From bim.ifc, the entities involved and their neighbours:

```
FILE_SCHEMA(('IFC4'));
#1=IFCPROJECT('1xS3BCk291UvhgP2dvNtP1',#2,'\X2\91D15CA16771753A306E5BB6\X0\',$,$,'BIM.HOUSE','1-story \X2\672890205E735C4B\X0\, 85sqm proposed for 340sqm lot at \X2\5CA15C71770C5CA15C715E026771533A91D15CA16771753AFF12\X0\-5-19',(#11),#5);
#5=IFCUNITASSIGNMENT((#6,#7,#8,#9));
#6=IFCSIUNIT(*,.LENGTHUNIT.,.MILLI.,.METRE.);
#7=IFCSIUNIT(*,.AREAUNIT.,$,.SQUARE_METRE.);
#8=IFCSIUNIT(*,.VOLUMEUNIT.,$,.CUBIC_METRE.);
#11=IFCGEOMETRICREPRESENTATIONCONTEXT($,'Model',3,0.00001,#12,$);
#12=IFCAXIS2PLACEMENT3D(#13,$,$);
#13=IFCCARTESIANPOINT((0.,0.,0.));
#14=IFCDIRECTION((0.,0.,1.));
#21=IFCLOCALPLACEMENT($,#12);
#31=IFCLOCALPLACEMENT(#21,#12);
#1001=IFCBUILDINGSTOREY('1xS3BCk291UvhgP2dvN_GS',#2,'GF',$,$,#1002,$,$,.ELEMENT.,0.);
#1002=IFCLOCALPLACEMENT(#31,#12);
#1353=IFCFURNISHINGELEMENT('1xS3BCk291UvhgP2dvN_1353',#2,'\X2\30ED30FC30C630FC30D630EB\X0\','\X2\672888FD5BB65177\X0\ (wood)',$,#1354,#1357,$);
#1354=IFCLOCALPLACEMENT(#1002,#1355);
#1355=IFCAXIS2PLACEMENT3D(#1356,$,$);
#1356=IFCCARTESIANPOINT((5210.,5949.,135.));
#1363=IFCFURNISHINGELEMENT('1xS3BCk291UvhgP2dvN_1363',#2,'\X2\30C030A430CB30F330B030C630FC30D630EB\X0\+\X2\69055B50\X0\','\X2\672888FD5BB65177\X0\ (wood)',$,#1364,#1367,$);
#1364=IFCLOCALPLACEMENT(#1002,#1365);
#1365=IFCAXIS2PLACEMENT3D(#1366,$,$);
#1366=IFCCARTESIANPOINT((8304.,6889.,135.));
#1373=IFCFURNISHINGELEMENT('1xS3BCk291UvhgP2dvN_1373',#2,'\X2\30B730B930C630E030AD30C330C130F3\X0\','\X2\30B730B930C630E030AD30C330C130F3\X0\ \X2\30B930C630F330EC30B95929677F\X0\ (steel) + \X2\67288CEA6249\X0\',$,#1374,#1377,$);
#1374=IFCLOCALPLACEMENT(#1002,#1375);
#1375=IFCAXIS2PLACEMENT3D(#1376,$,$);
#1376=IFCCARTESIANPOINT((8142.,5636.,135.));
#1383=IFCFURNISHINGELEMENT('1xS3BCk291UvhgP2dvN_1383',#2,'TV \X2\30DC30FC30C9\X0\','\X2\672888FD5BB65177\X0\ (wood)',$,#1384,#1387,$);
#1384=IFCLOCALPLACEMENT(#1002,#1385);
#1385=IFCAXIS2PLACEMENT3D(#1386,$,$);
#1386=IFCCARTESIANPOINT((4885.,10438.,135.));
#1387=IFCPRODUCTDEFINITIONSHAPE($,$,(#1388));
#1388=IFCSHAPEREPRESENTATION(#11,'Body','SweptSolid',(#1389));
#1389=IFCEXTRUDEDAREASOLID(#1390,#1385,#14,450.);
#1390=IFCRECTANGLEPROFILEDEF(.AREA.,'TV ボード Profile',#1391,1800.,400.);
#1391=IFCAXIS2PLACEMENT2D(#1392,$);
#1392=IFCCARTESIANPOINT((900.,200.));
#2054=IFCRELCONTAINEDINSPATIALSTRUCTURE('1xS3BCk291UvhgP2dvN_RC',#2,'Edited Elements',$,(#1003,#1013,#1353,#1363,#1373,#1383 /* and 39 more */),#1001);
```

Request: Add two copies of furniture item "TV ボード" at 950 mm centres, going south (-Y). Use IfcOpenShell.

```python
import numpy as np
import ifcopenshell
import ifcopenshell.api.geometry
import ifcopenshell.api.root
import ifcopenshell.util.element
import ifcopenshell.util.placement
import ifcopenshell.util.unit

model = ifcopenshell.open("bim.ifc")
unit_scale = ifcopenshell.util.unit.calculate_unit_scale(model)


def reuse_history(source, copy):
    """copy_class also copies each property set's owner history, people and application; keep the originals."""
    for rel in copy.IsDefinedBy:
        if rel.is_a("IfcRelDefinesByProperties") and (history := rel.RelatingPropertyDefinition.OwnerHistory):
            rel.RelatingPropertyDefinition.OwnerHistory = source.OwnerHistory
            ifcopenshell.util.element.remove_deep2(model, history)


source = model.by_guid("1xS3BCk291UvhgP2dvN_1383")
base = ifcopenshell.util.placement.get_local_placement(source.ObjectPlacement)
step = np.array([0.0, -1.0, 0.0]) * 0.95 / unit_scale

for i in range(1, 3):
    copy = ifcopenshell.api.root.copy_class(model, product=source)
    copy.Representation = ifcopenshell.util.element.copy_deep(
        model, source.Representation, exclude=["IfcGeometricRepresentationContext", "IfcRepresentationMap"]
    )
    reuse_history(source, copy)
    matrix = base.copy()
    matrix[:3, 3] += i * step
    print("added at", matrix[:3, 3].round(3) + 0.0)
    ifcopenshell.api.geometry.edit_object_placement(model, product=copy, matrix=matrix, is_si=False)

model.write("bim_edited.ifc")
```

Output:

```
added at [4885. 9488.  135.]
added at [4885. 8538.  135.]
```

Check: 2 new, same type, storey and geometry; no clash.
